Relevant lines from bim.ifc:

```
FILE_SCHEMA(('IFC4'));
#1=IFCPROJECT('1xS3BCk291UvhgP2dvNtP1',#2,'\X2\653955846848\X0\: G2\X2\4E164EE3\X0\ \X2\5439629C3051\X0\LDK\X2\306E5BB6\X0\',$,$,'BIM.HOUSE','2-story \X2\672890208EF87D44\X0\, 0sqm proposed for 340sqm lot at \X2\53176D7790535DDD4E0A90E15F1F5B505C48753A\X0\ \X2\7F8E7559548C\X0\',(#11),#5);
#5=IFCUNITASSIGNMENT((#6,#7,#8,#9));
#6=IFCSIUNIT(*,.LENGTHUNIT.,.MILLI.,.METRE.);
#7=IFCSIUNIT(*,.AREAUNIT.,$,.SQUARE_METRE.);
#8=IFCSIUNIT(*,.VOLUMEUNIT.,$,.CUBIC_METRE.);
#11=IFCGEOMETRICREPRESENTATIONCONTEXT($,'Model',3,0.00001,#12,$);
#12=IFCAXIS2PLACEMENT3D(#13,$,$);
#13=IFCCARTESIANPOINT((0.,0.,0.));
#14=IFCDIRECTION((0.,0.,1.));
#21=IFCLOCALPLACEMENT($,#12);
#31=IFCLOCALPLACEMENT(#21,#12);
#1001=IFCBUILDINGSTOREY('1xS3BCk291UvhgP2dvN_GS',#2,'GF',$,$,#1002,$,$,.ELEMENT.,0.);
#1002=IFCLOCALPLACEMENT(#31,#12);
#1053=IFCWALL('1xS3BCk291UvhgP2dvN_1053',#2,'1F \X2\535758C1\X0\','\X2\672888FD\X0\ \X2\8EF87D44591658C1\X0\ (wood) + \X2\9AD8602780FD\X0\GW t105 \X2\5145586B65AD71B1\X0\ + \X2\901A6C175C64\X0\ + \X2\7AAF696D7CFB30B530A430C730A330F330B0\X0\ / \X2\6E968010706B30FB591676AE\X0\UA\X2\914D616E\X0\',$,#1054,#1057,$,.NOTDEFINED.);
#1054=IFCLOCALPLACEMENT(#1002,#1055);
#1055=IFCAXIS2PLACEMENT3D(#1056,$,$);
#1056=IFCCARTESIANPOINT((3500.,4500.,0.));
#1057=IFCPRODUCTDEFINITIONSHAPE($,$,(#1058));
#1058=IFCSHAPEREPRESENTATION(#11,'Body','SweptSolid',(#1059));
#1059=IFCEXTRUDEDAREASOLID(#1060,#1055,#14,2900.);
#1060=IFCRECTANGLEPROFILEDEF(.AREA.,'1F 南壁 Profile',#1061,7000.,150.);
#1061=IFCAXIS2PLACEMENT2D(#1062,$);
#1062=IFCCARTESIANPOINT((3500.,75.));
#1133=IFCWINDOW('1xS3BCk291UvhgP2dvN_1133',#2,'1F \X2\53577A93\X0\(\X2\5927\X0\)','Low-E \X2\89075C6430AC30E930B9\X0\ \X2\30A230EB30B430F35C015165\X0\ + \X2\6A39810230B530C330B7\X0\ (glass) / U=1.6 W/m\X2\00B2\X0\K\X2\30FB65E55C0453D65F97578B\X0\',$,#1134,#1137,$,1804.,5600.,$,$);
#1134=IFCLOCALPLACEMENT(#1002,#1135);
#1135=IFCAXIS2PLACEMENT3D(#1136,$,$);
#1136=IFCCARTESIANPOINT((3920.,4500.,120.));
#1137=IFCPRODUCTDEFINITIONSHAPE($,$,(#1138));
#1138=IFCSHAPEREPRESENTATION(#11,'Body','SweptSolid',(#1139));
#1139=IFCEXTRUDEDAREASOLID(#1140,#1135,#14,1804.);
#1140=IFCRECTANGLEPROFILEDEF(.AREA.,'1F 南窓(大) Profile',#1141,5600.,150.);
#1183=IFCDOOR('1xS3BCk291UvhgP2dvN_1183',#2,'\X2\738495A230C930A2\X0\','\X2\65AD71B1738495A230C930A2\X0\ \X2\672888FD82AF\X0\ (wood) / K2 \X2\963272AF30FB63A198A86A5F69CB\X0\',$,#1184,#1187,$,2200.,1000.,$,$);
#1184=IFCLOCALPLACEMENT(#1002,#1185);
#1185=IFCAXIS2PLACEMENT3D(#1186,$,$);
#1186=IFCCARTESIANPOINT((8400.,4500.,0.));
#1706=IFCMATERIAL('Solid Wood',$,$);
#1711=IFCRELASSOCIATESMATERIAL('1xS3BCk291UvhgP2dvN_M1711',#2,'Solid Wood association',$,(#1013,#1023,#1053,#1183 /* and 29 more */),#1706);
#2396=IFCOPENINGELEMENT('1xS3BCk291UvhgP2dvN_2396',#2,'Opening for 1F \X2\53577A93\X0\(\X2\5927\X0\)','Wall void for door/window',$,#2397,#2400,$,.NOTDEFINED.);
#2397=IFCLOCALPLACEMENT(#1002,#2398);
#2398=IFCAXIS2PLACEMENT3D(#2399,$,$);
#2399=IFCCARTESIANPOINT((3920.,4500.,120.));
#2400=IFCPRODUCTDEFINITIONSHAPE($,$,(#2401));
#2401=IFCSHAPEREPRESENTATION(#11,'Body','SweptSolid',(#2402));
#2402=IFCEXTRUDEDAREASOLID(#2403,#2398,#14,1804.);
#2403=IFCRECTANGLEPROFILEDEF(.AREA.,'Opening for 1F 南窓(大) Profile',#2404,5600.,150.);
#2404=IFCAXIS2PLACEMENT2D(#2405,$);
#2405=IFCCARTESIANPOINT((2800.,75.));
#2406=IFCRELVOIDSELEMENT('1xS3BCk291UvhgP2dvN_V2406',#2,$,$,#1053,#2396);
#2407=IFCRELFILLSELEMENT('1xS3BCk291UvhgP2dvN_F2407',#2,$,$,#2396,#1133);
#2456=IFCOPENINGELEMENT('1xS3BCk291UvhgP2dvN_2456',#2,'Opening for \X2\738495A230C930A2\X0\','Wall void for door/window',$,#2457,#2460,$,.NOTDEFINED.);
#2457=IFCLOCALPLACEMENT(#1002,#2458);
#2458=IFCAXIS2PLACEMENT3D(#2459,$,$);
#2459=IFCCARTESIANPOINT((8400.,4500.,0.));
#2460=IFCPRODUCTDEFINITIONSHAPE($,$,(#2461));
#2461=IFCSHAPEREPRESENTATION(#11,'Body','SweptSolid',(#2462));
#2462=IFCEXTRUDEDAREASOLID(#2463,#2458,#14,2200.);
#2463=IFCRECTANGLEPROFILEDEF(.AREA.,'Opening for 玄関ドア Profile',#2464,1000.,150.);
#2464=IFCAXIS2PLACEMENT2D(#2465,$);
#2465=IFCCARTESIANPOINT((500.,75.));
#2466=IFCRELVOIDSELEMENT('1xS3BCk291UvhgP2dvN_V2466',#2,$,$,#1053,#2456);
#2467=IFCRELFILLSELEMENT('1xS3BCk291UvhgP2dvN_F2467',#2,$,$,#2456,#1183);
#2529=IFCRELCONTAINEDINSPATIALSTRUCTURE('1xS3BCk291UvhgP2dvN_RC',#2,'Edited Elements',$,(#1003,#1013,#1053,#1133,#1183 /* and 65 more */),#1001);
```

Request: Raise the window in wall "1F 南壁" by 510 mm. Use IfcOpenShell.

```python
import numpy as np
import ifcopenshell
import ifcopenshell.api.geometry
import ifcopenshell.util.placement
import ifcopenshell.util.unit

model = ifcopenshell.open("bim.ifc")
unit_scale = ifcopenshell.util.unit.calculate_unit_scale(model)

window = model.by_guid("1xS3BCk291UvhgP2dvN_1133")
opening = window.FillsVoids[0].RelatingOpeningElement
dz = 510.0

shift = np.array([0.0, 0.0, dz])
# The window is not placed relative to its opening, so move both.
for product in (opening, window):
    matrix = ifcopenshell.util.placement.get_local_placement(product.ObjectPlacement)
    matrix[:3, 3] += shift
    ifcopenshell.api.geometry.edit_object_placement(model, product=product, matrix=matrix, is_si=False)

print(f"moved by {dz * unit_scale:+.3f} m")

model.write("bim_rev.ifc")
```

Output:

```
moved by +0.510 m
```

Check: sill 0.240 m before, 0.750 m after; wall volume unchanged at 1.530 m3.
